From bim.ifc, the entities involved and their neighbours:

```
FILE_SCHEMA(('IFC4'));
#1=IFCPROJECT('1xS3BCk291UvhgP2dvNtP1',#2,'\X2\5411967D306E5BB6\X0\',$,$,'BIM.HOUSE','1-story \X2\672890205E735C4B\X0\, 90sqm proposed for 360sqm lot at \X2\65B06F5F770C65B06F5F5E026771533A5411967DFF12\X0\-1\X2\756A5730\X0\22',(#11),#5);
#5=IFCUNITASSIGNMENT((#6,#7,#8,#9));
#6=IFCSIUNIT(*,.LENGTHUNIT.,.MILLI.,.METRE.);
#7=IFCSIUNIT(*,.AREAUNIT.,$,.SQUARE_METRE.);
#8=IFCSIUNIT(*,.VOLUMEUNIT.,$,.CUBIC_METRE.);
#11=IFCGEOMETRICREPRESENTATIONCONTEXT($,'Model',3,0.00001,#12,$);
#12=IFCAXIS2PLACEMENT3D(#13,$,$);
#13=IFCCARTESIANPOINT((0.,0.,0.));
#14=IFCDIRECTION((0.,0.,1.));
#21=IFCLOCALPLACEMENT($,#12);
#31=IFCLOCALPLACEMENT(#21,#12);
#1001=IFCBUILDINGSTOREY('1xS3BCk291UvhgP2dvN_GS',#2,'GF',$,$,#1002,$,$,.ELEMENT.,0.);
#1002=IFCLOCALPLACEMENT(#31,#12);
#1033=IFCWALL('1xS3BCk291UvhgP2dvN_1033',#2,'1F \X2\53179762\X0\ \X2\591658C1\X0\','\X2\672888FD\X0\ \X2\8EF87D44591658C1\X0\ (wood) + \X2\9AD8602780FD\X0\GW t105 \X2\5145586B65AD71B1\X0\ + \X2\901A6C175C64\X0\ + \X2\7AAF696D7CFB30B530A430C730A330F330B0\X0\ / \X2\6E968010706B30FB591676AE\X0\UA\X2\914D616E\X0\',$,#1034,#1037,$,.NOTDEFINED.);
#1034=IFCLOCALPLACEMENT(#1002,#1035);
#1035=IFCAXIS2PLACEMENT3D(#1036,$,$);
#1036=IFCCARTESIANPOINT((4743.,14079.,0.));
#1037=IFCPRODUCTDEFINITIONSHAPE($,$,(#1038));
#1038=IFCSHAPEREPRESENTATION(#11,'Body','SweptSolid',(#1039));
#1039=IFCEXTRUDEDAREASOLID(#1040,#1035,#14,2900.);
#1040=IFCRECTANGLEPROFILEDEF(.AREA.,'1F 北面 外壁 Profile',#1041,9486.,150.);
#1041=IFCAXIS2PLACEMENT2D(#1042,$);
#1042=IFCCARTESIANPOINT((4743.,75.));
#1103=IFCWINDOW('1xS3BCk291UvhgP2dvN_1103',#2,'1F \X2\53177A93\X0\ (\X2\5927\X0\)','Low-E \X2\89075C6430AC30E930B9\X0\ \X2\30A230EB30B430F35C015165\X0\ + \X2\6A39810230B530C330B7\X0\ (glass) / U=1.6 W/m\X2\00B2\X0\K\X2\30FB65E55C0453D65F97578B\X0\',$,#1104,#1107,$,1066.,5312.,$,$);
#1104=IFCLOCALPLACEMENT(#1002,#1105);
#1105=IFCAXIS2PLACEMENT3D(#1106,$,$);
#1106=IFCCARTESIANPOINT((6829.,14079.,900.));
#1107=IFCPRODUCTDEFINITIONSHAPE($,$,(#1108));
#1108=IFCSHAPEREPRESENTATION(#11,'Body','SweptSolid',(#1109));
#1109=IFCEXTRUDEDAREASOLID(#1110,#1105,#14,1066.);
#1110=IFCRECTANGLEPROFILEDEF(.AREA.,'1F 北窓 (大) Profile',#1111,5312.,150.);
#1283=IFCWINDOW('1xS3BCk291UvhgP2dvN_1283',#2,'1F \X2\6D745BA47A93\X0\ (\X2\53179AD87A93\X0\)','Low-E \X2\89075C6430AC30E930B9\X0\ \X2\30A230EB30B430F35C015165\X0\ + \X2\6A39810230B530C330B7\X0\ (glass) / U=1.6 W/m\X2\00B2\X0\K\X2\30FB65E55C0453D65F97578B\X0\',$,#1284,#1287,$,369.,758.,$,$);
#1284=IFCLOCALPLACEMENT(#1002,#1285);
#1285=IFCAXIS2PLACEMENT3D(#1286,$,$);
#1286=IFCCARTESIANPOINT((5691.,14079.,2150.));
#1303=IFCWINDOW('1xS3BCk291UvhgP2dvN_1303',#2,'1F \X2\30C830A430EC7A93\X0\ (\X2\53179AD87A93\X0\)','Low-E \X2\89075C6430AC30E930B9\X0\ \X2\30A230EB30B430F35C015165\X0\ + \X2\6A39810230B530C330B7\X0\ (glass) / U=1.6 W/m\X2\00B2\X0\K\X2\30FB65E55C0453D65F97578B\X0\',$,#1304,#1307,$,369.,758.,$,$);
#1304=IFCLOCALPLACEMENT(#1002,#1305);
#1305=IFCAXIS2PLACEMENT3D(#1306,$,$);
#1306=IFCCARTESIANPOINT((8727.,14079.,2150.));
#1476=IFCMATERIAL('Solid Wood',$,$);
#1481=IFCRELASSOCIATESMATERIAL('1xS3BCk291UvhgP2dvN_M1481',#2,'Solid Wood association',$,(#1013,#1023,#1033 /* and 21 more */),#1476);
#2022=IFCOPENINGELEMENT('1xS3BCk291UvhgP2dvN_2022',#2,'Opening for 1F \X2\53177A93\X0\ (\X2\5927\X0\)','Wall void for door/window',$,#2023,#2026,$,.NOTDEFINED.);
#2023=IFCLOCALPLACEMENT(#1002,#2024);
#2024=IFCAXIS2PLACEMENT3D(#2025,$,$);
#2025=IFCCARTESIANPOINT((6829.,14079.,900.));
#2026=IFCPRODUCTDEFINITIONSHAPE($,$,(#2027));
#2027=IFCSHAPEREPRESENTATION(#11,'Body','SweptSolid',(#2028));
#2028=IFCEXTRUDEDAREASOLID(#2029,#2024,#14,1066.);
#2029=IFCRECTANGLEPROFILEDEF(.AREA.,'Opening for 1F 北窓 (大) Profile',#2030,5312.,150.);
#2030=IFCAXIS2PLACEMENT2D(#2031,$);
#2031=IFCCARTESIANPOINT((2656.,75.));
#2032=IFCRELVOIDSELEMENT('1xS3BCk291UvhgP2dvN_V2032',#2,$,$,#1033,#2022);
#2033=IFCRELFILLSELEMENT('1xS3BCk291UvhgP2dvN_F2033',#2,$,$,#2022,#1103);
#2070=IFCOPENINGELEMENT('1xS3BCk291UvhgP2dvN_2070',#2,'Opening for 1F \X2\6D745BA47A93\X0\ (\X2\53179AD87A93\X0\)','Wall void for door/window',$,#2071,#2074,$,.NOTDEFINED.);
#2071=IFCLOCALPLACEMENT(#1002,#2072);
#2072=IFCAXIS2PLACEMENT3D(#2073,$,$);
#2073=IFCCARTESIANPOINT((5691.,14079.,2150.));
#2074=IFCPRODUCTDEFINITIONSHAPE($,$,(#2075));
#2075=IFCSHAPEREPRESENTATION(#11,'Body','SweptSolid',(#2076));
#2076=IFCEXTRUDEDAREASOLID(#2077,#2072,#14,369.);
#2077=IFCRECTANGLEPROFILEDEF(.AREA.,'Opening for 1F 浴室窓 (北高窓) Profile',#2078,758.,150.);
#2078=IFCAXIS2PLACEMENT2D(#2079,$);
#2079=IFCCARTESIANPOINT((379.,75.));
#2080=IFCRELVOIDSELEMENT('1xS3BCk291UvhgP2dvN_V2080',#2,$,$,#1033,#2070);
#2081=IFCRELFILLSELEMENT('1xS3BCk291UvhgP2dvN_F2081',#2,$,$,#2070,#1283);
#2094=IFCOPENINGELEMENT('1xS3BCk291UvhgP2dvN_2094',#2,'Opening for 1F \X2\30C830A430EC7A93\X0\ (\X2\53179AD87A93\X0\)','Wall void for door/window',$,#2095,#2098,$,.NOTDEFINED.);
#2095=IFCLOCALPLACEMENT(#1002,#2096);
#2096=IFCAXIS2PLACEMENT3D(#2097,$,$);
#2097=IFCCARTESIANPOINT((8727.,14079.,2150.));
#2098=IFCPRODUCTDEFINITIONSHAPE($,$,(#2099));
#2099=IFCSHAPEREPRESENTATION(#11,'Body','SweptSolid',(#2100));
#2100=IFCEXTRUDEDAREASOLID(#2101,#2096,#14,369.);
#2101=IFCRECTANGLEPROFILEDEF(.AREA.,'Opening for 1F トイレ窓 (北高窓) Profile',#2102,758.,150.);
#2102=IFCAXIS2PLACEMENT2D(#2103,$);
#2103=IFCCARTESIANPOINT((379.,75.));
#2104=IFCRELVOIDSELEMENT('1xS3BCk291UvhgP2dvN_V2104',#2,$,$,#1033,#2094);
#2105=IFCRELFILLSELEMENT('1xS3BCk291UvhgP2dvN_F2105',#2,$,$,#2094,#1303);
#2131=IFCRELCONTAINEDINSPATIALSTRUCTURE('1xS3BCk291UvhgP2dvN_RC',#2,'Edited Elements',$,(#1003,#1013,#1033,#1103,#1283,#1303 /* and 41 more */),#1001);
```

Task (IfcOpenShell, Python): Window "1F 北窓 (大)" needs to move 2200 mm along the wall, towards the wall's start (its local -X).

```python
import ifcopenshell
import ifcopenshell.api.geometry
import ifcopenshell.util.placement

model = ifcopenshell.open("bim.ifc")

window = model.by_guid("1xS3BCk291UvhgP2dvN_1103")
opening = window.FillsVoids[0].RelatingOpeningElement
wall = opening.VoidsElements[0].RelatingBuildingElement

wall_matrix = ifcopenshell.util.placement.get_local_placement(wall.ObjectPlacement)
shift = wall_matrix[:3, 0] * -2200.0
before = ifcopenshell.util.placement.get_local_placement(window.ObjectPlacement)[:3, 3].copy()

# The window is not placed relative to its opening, so move both.
for product in (opening, window):
    matrix = ifcopenshell.util.placement.get_local_placement(product.ObjectPlacement)
    matrix[:3, 3] += shift
    ifcopenshell.api.geometry.edit_object_placement(model, product=product, matrix=matrix, is_si=False)

after = ifcopenshell.util.placement.get_local_placement(window.ObjectPlacement)[:3, 3]
print("window moved by", (after - before).round(3) + 0.0)

model.write("bim_updated.ifc")
```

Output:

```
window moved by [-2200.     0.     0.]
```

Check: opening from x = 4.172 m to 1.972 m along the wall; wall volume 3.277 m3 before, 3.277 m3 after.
